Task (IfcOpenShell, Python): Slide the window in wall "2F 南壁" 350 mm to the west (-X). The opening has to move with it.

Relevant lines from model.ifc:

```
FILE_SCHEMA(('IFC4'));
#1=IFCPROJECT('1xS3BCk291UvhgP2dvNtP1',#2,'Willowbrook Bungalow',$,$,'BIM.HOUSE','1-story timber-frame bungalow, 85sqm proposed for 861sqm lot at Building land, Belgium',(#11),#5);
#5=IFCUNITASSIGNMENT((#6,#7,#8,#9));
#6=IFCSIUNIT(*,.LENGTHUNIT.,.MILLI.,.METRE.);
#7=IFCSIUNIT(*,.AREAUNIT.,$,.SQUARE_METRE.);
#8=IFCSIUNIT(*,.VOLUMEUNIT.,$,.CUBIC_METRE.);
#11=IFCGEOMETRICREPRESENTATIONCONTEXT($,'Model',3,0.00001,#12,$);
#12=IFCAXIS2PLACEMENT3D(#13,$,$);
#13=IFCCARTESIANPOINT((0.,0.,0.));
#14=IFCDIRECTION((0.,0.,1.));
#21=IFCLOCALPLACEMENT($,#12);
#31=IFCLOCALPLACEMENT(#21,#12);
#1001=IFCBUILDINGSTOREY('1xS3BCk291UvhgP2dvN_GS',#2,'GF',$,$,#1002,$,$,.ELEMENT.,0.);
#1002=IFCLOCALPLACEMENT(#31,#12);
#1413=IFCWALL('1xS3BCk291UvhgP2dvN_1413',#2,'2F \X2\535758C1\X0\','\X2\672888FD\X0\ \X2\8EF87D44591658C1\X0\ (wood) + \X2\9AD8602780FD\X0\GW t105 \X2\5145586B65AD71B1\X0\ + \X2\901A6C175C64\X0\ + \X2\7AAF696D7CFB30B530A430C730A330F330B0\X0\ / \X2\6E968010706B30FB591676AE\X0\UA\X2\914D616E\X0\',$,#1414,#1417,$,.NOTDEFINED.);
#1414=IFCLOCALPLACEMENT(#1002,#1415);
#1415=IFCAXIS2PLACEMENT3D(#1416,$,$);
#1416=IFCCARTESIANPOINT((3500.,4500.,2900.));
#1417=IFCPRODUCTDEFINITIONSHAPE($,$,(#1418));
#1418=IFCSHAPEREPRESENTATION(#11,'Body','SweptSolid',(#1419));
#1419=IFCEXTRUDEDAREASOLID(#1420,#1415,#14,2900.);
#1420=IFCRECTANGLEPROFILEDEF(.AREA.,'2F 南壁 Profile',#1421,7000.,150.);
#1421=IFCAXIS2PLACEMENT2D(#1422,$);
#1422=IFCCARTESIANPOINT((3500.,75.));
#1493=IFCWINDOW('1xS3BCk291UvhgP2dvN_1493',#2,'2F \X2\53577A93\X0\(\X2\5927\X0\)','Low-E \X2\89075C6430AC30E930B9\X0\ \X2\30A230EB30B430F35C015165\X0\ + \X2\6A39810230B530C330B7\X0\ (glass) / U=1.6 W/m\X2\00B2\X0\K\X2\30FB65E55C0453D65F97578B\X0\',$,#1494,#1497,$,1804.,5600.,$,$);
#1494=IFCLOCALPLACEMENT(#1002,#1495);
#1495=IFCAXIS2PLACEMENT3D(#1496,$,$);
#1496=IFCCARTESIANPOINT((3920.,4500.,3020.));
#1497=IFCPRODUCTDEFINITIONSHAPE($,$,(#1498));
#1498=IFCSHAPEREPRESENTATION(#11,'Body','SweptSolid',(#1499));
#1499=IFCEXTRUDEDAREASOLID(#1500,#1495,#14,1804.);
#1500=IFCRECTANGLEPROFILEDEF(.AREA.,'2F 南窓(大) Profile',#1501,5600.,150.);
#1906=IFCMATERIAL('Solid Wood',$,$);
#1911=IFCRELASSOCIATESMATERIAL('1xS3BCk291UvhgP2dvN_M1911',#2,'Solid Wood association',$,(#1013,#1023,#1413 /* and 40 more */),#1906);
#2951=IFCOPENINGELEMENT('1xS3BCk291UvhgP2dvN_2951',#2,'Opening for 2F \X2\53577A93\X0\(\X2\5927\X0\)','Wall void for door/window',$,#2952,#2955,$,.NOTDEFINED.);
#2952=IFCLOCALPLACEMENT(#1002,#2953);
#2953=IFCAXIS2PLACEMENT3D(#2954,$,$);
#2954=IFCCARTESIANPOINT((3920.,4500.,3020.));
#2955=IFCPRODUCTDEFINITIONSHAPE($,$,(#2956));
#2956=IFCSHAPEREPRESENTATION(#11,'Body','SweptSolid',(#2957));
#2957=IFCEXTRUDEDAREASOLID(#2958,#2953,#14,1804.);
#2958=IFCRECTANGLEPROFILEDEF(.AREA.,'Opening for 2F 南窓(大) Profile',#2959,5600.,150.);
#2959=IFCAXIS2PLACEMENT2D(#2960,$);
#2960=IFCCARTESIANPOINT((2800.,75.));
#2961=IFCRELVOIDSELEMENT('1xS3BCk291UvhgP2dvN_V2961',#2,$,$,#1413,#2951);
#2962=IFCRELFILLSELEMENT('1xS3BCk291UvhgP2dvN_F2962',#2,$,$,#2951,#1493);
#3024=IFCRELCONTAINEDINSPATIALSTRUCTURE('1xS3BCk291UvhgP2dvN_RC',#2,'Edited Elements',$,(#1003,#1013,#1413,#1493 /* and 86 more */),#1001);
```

```python
import ifcopenshell
import ifcopenshell.api.geometry
import ifcopenshell.util.placement

model = ifcopenshell.open("model.ifc")

window = model.by_id(1493)
opening = window.FillsVoids[0].RelatingOpeningElement
wall = opening.VoidsElements[0].RelatingBuildingElement

wall_matrix = ifcopenshell.util.placement.get_local_placement(wall.ObjectPlacement)
shift = wall_matrix[:3, 0] * -350.0
before = ifcopenshell.util.placement.get_local_placement(window.ObjectPlacement)[:3, 3].copy()

# The window is not placed relative to its opening, so move both.
for product in (opening, window):
    matrix = ifcopenshell.util.placement.get_local_placement(product.ObjectPlacement)
    matrix[:3, 3] += shift
    ifcopenshell.api.geometry.edit_object_placement(model, product=product, matrix=matrix, is_si=False)

after = ifcopenshell.util.placement.get_local_placement(window.ObjectPlacement)[:3, 3]
print("window moved by", (after - before).round(3) + 0.0)

model.write("model_updated.ifc")
```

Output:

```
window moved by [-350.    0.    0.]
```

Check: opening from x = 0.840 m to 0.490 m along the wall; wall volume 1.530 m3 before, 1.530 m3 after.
